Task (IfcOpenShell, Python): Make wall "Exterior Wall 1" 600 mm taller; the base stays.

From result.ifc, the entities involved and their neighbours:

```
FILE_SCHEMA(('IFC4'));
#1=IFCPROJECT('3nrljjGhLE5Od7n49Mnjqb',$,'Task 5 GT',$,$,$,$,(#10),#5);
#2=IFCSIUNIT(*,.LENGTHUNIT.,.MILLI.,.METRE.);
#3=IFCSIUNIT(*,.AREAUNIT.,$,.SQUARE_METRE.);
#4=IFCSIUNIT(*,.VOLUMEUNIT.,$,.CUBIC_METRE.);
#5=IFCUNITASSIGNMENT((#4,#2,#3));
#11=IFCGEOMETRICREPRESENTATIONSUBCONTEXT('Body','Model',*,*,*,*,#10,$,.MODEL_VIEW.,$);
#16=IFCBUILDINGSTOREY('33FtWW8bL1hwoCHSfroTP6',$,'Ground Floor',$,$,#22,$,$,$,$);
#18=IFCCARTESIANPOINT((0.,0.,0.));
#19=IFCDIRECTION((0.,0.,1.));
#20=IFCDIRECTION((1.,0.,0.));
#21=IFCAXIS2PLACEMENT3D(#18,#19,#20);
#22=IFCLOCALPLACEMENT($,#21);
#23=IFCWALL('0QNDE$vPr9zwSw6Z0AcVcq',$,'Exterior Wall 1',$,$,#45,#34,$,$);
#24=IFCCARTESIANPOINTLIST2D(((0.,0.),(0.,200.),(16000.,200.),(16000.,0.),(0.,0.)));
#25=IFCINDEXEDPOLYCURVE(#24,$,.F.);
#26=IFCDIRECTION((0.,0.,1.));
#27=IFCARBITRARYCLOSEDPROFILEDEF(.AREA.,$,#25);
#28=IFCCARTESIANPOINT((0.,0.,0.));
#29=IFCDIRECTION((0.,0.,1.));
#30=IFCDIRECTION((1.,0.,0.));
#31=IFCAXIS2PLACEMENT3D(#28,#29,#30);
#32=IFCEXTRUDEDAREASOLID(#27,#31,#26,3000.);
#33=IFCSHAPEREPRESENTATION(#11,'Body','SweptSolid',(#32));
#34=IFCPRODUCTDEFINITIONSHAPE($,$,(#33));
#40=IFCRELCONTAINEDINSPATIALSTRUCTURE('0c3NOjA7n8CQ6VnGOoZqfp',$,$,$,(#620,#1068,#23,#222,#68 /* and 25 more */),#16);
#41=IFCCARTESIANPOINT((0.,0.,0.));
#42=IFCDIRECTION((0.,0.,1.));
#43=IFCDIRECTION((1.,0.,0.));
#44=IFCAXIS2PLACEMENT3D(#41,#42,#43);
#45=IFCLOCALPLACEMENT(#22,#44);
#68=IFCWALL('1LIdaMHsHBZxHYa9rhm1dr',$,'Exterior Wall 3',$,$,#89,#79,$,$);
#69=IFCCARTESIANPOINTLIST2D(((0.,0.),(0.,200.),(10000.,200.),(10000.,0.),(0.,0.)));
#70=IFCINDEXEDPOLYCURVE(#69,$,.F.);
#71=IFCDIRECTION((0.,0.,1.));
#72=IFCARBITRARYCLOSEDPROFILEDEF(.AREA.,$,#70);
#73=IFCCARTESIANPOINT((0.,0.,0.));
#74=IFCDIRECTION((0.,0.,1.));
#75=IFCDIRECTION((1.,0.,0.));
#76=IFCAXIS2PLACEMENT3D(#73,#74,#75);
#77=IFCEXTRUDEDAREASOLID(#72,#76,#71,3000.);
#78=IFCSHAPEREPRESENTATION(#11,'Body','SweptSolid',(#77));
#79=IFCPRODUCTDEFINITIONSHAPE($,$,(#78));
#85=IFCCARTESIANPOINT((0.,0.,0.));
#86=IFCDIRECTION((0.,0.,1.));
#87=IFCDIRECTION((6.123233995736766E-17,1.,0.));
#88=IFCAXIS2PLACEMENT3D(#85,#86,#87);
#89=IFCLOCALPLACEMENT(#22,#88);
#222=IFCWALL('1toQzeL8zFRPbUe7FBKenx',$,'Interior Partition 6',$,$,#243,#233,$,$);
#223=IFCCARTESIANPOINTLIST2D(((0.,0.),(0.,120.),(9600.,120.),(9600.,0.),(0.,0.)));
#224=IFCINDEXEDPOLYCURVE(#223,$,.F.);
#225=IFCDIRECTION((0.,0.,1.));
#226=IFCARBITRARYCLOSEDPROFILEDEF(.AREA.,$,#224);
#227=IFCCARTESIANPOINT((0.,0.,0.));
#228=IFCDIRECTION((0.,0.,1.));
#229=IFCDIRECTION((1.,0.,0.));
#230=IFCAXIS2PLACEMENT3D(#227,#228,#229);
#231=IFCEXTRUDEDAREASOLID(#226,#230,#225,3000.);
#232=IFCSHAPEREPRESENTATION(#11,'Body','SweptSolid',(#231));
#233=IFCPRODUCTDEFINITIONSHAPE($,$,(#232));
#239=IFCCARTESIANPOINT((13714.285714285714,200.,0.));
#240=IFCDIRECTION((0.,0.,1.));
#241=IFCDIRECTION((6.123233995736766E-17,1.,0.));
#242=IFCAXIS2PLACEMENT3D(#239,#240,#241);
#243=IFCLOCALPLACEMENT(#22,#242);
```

```python
import ifcopenshell
import ifcopenshell.geom
import ifcopenshell.util.representation
import ifcopenshell.util.shape

model = ifcopenshell.open("result.ifc")
settings = ifcopenshell.geom.settings()


def volume(element):
    """Net volume in cubic metres, openings subtracted."""
    shape = ifcopenshell.geom.create_shape(settings, element)
    return ifcopenshell.util.shape.get_volume(shape.geometry)


wall = model.by_guid("0QNDE$vPr9zwSw6Z0AcVcq")
before = volume(wall)

body = ifcopenshell.util.representation.get_representation(wall, "Model", "Body")
solid = body.Items[0]
old_height = solid.Depth
solid.Depth += 600.0
after = volume(wall)

print(f"height {old_height:g} -> {solid.Depth:g}, volume {before:.3f} -> {after:.3f} m3")

model.write("result-out.ifc")
```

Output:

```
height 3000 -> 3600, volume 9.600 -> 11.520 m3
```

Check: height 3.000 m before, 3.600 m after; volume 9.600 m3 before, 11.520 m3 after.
